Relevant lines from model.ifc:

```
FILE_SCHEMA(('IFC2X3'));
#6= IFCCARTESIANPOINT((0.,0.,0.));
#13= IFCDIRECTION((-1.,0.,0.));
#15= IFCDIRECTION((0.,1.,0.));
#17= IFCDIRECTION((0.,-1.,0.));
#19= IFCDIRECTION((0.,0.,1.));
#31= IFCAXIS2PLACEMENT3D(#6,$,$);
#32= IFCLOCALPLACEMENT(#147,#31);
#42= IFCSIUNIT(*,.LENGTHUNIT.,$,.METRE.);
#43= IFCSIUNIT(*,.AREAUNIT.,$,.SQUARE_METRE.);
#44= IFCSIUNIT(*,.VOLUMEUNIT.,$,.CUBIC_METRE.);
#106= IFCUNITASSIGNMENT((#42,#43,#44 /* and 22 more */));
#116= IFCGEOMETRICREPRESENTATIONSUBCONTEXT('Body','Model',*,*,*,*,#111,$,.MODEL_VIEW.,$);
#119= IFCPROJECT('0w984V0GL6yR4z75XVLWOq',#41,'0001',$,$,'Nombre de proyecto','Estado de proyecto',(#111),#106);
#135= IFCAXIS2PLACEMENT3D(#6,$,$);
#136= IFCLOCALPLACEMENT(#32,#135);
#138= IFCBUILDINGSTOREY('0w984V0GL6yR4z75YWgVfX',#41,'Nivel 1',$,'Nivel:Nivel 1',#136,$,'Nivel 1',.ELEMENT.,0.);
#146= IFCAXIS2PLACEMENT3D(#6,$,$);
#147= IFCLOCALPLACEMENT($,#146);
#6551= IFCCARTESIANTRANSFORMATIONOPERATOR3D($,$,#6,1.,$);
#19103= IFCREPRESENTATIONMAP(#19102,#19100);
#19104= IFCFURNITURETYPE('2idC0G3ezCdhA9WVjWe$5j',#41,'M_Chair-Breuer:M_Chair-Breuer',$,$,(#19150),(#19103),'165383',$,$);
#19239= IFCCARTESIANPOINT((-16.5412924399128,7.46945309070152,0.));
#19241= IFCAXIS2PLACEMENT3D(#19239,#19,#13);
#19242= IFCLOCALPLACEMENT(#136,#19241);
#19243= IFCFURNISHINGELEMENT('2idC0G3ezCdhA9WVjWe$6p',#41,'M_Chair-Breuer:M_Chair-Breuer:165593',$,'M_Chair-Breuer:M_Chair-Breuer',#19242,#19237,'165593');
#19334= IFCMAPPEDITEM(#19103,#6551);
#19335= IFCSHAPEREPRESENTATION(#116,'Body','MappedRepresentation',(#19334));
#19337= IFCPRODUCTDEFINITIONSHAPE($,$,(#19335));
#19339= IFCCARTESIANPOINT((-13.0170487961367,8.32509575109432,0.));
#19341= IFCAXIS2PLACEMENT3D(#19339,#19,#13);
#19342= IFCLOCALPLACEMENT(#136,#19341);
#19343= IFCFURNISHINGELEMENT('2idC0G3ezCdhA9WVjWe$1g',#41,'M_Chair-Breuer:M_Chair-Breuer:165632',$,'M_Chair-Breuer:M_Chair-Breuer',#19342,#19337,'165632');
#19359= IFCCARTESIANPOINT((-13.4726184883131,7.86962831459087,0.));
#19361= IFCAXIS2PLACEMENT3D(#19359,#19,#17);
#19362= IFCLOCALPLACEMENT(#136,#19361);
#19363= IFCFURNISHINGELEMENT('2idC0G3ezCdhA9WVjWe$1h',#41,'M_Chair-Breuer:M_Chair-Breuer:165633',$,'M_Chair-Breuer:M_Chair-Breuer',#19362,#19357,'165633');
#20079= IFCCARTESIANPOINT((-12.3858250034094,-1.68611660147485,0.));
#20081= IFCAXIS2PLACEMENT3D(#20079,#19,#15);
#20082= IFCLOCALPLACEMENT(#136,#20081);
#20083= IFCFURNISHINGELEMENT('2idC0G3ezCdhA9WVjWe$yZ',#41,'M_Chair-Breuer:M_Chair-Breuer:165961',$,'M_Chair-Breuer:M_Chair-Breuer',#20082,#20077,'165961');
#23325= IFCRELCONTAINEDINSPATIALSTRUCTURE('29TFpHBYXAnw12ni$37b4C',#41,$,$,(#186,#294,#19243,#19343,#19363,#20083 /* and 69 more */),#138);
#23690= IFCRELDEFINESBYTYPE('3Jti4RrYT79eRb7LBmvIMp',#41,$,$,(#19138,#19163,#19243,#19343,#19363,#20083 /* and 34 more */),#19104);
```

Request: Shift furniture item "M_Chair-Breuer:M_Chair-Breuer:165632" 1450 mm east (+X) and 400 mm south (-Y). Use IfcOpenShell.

```python
import ifcopenshell
import ifcopenshell.api.geometry
import ifcopenshell.util.placement
import ifcopenshell.util.unit

model = ifcopenshell.open("model.ifc")
unit_scale = ifcopenshell.util.unit.calculate_unit_scale(model)

item = model.by_guid("2idC0G3ezCdhA9WVjWe$1g")
matrix = ifcopenshell.util.placement.get_local_placement(item.ObjectPlacement)
matrix[0, 3] += 1.45 / unit_scale
matrix[1, 3] -= 0.4 / unit_scale
ifcopenshell.api.geometry.edit_object_placement(model, product=item, matrix=matrix, is_si=False)

print(ifcopenshell.util.placement.get_local_placement(item.ObjectPlacement).round(3) + 0.0)

model.write("model_v2.ifc")
```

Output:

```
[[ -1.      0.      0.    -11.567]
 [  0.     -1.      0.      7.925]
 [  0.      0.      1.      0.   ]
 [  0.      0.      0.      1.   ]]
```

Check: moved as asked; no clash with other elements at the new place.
